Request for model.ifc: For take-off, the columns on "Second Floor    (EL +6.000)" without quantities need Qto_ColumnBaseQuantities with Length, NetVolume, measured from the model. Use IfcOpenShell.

First a look at what the model holds.

```python
import ifcopenshell
import ifcopenshell.util.element
import ifcopenshell.util.unit

model = ifcopenshell.open("model.ifc")
print(model.schema)
for unit_type in ("LENGTHUNIT", "AREAUNIT", "VOLUMEUNIT"):
    print(unit_type, ifcopenshell.util.unit.calculate_unit_scale(model, unit_type))
storey = next(s for s in model.by_type("IfcBuildingStorey") if s.Name == "Second Floor    (EL +6.000)")
columns = [e for e in ifcopenshell.util.element.get_decomposition(storey) if e.is_a("IfcColumn")]
for e in sorted(columns, key=lambda e: e.id()):
    print(e.id(), e.is_a(), e.Name, list(ifcopenshell.util.element.get_psets(e, qtos_only=True)), sep=" | ")
```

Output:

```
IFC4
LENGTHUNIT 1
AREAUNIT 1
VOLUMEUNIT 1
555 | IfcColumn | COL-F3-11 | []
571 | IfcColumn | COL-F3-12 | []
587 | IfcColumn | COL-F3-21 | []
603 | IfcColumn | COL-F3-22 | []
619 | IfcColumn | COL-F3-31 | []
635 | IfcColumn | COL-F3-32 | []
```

```python
import ifcopenshell
import ifcopenshell.api.pset
import ifcopenshell.geom
import ifcopenshell.util.element
import ifcopenshell.util.shape
import ifcopenshell.util.unit

model = ifcopenshell.open("model.ifc")
unit_scale = ifcopenshell.util.unit.calculate_unit_scale(model)
volume_scale = ifcopenshell.util.unit.calculate_unit_scale(model, "VOLUMEUNIT")
settings = ifcopenshell.geom.settings()

storey = next(s for s in model.by_type("IfcBuildingStorey") if s.Name == "Second Floor    (EL +6.000)")
columns = [e for e in ifcopenshell.util.element.get_decomposition(storey) if e.is_a("IfcColumn")]

for e in sorted(columns, key=lambda e: e.id()):
    if ifcopenshell.util.element.get_psets(e, qtos_only=True, should_inherit=False):
        continue
    # Geometry comes back in metres, in the element's own axes.
    shape = ifcopenshell.geom.create_shape(settings, e)
    values = {
        "Length": ifcopenshell.util.shape.get_z(shape.geometry) / unit_scale,
        "NetVolume": ifcopenshell.util.shape.get_volume(shape.geometry) / volume_scale,
    }
    qto = ifcopenshell.api.pset.add_qto(model, product=e, name="Qto_ColumnBaseQuantities")
    ifcopenshell.api.pset.edit_qto(model, qto=qto, properties=values)
    print(e.id(), {k: round(v, 3) for k, v in values.items()})

model.write("model_updated.ifc")
```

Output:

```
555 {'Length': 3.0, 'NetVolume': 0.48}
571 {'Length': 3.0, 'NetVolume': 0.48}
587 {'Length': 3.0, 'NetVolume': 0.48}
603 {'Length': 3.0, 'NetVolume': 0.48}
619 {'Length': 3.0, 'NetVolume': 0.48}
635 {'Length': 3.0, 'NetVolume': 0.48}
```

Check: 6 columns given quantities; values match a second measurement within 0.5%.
